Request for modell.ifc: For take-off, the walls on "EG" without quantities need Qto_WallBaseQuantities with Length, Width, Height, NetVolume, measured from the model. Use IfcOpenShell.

First a look at what the model holds.

```python
import ifcopenshell
import ifcopenshell.util.element
import ifcopenshell.util.unit

model = ifcopenshell.open("modell.ifc")
print(model.schema)
for unit_type in ("LENGTHUNIT", "AREAUNIT", "VOLUMEUNIT"):
    print(unit_type, ifcopenshell.util.unit.calculate_unit_scale(model, unit_type))
storey = next(s for s in model.by_type("IfcBuildingStorey") if s.Name == "EG")
walls = [e for e in ifcopenshell.util.element.get_decomposition(storey) if e.is_a("IfcWall")]
for e in sorted(walls, key=lambda e: e.id()):
    print(e.id(), e.is_a(), e.Name, list(ifcopenshell.util.element.get_psets(e, qtos_only=True)), sep=" | ")
```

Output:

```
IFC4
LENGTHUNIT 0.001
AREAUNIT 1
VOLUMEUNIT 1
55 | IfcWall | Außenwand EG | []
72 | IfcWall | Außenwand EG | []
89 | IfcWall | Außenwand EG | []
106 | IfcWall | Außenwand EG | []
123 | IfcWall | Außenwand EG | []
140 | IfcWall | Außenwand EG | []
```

```python
import ifcopenshell
import ifcopenshell.api.pset
import ifcopenshell.geom
import ifcopenshell.util.element
import ifcopenshell.util.shape
import ifcopenshell.util.unit

model = ifcopenshell.open("modell.ifc")
unit_scale = ifcopenshell.util.unit.calculate_unit_scale(model)
volume_scale = ifcopenshell.util.unit.calculate_unit_scale(model, "VOLUMEUNIT")
settings = ifcopenshell.geom.settings()

storey = next(s for s in model.by_type("IfcBuildingStorey") if s.Name == "EG")
walls = [e for e in ifcopenshell.util.element.get_decomposition(storey) if e.is_a("IfcWall")]

for e in sorted(walls, key=lambda e: e.id()):
    if ifcopenshell.util.element.get_psets(e, qtos_only=True, should_inherit=False):
        continue
    # Geometry comes back in metres, in the element's own axes.
    shape = ifcopenshell.geom.create_shape(settings, e)
    values = {
        "Length": ifcopenshell.util.shape.get_x(shape.geometry) / unit_scale,
        "Width": ifcopenshell.util.shape.get_y(shape.geometry) / unit_scale,
        "Height": ifcopenshell.util.shape.get_z(shape.geometry) / unit_scale,
        "NetVolume": ifcopenshell.util.shape.get_volume(shape.geometry) / volume_scale,
    }
    qto = ifcopenshell.api.pset.add_qto(model, product=e, name="Qto_WallBaseQuantities")
    ifcopenshell.api.pset.edit_qto(model, qto=qto, properties=values)
    print(e.id(), {k: round(v, 3) for k, v in values.items()})

model.write("modell_rev.ifc")
```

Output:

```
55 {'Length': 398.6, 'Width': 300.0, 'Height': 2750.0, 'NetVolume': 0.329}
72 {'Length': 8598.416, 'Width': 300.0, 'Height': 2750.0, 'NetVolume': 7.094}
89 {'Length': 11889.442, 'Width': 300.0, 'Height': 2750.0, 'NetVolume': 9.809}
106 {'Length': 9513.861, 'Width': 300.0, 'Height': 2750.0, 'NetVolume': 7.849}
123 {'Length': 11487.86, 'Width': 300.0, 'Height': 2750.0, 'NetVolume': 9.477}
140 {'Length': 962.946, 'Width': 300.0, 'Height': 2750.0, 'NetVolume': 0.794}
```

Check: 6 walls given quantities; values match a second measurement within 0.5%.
